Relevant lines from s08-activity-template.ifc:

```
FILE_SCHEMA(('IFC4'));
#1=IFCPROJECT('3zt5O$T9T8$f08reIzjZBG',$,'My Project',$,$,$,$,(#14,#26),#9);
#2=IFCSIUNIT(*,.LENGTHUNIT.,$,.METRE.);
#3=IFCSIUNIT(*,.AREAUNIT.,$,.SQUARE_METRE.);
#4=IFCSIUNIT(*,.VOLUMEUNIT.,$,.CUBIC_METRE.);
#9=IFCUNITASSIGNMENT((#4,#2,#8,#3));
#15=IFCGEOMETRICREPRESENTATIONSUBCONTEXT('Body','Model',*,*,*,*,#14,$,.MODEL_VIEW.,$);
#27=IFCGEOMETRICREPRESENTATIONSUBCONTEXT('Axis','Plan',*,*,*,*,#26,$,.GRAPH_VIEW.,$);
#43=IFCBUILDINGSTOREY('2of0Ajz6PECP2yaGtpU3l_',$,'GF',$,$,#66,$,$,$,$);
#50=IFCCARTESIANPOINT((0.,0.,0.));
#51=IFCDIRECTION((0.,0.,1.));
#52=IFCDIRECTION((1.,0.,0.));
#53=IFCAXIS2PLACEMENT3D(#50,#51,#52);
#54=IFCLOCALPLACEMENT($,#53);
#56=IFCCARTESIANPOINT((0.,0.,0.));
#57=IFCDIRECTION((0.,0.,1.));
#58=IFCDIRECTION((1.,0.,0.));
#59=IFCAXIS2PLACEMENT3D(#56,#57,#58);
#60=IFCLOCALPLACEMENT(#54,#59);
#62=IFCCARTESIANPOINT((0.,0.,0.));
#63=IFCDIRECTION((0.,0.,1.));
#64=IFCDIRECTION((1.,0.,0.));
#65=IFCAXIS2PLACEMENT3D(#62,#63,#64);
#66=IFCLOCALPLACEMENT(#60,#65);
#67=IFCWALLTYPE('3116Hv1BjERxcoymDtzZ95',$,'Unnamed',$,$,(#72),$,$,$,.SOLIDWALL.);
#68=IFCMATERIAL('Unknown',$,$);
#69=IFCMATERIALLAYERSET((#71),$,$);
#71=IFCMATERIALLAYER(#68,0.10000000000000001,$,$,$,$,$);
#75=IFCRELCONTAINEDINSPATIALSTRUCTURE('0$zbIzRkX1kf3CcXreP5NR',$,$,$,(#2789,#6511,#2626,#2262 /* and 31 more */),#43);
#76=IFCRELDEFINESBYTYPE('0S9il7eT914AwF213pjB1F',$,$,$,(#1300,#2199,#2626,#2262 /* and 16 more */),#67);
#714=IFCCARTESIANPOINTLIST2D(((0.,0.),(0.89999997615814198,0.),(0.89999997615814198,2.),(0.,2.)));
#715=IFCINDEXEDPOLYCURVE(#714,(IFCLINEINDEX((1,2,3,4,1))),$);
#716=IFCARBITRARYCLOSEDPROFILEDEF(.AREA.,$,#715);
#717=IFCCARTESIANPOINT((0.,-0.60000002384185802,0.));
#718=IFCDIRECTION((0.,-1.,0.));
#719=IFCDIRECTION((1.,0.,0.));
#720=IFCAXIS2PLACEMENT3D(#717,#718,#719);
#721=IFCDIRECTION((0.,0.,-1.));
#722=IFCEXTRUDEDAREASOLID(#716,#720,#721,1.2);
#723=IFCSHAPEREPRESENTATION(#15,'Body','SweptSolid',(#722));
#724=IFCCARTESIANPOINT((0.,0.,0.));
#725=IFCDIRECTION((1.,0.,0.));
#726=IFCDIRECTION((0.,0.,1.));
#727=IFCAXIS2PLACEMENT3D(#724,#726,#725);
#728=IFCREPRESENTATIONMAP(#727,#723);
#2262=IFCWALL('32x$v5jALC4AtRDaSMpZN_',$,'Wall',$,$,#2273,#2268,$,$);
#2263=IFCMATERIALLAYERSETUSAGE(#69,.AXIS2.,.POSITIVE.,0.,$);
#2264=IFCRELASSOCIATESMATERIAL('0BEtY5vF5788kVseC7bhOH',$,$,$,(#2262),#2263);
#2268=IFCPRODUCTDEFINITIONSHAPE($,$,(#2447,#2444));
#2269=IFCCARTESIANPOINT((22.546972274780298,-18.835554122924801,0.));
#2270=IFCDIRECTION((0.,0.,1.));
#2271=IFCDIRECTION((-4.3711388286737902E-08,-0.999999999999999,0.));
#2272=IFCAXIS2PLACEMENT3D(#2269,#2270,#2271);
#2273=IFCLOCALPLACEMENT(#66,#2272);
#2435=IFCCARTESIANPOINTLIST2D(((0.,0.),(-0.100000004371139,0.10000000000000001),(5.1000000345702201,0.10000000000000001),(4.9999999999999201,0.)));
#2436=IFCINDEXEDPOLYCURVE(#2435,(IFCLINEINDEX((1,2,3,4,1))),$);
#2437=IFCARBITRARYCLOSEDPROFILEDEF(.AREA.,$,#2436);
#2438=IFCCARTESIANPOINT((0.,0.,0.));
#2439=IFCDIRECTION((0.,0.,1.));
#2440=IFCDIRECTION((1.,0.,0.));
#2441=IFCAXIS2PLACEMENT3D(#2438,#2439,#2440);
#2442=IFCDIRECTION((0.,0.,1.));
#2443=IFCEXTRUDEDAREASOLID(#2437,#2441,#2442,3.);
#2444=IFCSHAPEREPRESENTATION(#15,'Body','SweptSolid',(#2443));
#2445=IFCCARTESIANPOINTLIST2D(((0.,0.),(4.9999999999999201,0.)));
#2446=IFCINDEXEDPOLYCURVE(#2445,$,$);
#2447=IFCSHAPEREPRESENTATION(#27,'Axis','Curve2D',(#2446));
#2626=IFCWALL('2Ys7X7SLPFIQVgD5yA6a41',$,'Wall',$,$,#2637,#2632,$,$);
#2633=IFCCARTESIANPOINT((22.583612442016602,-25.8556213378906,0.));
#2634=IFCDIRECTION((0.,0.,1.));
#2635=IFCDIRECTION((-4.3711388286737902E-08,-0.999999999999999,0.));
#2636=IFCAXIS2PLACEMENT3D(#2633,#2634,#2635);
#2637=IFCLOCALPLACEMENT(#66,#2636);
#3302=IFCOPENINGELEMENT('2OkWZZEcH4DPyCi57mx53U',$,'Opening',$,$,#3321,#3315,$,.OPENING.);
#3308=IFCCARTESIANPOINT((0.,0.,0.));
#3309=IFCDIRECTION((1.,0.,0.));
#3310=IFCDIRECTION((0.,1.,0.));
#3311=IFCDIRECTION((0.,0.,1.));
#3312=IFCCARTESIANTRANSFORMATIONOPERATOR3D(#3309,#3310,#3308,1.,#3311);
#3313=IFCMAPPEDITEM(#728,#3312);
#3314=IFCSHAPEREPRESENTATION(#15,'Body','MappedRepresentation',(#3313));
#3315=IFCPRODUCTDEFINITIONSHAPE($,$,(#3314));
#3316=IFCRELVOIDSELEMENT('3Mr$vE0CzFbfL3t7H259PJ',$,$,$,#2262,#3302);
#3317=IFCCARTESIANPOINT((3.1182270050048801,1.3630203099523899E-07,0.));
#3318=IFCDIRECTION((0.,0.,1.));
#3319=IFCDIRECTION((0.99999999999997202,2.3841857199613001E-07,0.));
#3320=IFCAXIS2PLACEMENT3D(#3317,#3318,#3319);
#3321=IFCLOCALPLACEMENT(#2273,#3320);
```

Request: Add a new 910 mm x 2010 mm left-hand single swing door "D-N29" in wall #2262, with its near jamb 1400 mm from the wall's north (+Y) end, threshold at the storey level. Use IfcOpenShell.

```python
import numpy as np
import ifcopenshell
import ifcopenshell.api.feature
import ifcopenshell.api.geometry
import ifcopenshell.api.root
import ifcopenshell.api.spatial
import ifcopenshell.geom
import ifcopenshell.util.element
import ifcopenshell.util.placement
import ifcopenshell.util.representation
import ifcopenshell.util.shape
import ifcopenshell.util.unit

model = ifcopenshell.open("s08-activity-template.ifc")
unit_scale = ifcopenshell.util.unit.calculate_unit_scale(model)
settings = ifcopenshell.geom.settings()


def volume(element):
    """Net volume in cubic metres, openings subtracted."""
    shape = ifcopenshell.geom.create_shape(settings, element)
    return ifcopenshell.util.shape.get_volume(shape.geometry)


wall = model.by_guid("32x$v5jALC4AtRDaSMpZN_")
storey = ifcopenshell.util.element.get_container(wall, ifc_class="IfcBuildingStorey")
context = ifcopenshell.util.representation.get_context(model, "Model", "Body", "MODEL_VIEW")
before = volume(wall)

width, height, from_end, sill = 0.91, 2.01, 1.4, 0.0  # metres

# The wall runs along its own X axis, and the end named is its -X end.
wall_shape = ifcopenshell.geom.create_shape(settings, wall)
x, y, z = ifcopenshell.util.shape.get_vertices(wall_shape.geometry).T
start = x.min() + from_end
face, thickness = float(y.min()), float(y.max() - y.min())
wall_matrix = ifcopenshell.util.placement.get_local_placement(wall.ObjectPlacement)
level = ifcopenshell.util.placement.get_local_placement(storey.ObjectPlacement)[2, 3]


def in_wall(x, y):
    """Placement at x, y metres in the wall's axes, at sill height."""
    matrix = wall_matrix.copy()
    matrix[:, 3] = wall_matrix @ np.array([x / unit_scale, y / unit_scale, 0.0, 1.0])
    matrix[2, 3] = level + sill / unit_scale
    return matrix


# Opening: a box that overshoots both wall faces by 50 mm.
opening = ifcopenshell.api.root.create_entity(model, ifc_class="IfcOpeningElement", predefined_type="OPENING")
box = ifcopenshell.api.geometry.add_wall_representation(
    model, context=context, length=width, height=height, thickness=thickness + 0.1
)
ifcopenshell.api.geometry.assign_representation(model, product=opening, representation=box)
ifcopenshell.api.geometry.edit_object_placement(model, product=opening, matrix=in_wall(start, face - 0.05), is_si=False)
ifcopenshell.api.feature.add_feature(model, feature=opening, element=wall)

door = ifcopenshell.api.root.create_entity(model, ifc_class="IfcDoor", name="D-N29", predefined_type="DOOR")
door.OverallWidth, door.OverallHeight = width / unit_scale, height / unit_scale
door.OperationType = "SINGLE_SWING_LEFT"
body = ifcopenshell.api.geometry.add_door_representation(
    model,
    context=context,
    overall_width=door.OverallWidth,
    overall_height=door.OverallHeight,
    operation_type="SINGLE_SWING_LEFT",
    lining_properties={"LiningDepth": thickness / unit_scale, "ThresholdDepth": thickness / unit_scale},
)
ifcopenshell.api.geometry.assign_representation(model, product=door, representation=body)
ifcopenshell.api.spatial.assign_container(model, products=[door], relating_structure=storey)
ifcopenshell.api.feature.add_filling(model, opening=opening, element=door)

# The lining spans the wall, so the door starts at the wall face.
ifcopenshell.api.geometry.edit_object_placement(model, product=door, matrix=in_wall(start, face), is_si=False)

after = volume(wall)

print(f"wall volume {before:.3f} -> {after:.3f} m3")

model.write("s08-activity-template_v2.ifc")
```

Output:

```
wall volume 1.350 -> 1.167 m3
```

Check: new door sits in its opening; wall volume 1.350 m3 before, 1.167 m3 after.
